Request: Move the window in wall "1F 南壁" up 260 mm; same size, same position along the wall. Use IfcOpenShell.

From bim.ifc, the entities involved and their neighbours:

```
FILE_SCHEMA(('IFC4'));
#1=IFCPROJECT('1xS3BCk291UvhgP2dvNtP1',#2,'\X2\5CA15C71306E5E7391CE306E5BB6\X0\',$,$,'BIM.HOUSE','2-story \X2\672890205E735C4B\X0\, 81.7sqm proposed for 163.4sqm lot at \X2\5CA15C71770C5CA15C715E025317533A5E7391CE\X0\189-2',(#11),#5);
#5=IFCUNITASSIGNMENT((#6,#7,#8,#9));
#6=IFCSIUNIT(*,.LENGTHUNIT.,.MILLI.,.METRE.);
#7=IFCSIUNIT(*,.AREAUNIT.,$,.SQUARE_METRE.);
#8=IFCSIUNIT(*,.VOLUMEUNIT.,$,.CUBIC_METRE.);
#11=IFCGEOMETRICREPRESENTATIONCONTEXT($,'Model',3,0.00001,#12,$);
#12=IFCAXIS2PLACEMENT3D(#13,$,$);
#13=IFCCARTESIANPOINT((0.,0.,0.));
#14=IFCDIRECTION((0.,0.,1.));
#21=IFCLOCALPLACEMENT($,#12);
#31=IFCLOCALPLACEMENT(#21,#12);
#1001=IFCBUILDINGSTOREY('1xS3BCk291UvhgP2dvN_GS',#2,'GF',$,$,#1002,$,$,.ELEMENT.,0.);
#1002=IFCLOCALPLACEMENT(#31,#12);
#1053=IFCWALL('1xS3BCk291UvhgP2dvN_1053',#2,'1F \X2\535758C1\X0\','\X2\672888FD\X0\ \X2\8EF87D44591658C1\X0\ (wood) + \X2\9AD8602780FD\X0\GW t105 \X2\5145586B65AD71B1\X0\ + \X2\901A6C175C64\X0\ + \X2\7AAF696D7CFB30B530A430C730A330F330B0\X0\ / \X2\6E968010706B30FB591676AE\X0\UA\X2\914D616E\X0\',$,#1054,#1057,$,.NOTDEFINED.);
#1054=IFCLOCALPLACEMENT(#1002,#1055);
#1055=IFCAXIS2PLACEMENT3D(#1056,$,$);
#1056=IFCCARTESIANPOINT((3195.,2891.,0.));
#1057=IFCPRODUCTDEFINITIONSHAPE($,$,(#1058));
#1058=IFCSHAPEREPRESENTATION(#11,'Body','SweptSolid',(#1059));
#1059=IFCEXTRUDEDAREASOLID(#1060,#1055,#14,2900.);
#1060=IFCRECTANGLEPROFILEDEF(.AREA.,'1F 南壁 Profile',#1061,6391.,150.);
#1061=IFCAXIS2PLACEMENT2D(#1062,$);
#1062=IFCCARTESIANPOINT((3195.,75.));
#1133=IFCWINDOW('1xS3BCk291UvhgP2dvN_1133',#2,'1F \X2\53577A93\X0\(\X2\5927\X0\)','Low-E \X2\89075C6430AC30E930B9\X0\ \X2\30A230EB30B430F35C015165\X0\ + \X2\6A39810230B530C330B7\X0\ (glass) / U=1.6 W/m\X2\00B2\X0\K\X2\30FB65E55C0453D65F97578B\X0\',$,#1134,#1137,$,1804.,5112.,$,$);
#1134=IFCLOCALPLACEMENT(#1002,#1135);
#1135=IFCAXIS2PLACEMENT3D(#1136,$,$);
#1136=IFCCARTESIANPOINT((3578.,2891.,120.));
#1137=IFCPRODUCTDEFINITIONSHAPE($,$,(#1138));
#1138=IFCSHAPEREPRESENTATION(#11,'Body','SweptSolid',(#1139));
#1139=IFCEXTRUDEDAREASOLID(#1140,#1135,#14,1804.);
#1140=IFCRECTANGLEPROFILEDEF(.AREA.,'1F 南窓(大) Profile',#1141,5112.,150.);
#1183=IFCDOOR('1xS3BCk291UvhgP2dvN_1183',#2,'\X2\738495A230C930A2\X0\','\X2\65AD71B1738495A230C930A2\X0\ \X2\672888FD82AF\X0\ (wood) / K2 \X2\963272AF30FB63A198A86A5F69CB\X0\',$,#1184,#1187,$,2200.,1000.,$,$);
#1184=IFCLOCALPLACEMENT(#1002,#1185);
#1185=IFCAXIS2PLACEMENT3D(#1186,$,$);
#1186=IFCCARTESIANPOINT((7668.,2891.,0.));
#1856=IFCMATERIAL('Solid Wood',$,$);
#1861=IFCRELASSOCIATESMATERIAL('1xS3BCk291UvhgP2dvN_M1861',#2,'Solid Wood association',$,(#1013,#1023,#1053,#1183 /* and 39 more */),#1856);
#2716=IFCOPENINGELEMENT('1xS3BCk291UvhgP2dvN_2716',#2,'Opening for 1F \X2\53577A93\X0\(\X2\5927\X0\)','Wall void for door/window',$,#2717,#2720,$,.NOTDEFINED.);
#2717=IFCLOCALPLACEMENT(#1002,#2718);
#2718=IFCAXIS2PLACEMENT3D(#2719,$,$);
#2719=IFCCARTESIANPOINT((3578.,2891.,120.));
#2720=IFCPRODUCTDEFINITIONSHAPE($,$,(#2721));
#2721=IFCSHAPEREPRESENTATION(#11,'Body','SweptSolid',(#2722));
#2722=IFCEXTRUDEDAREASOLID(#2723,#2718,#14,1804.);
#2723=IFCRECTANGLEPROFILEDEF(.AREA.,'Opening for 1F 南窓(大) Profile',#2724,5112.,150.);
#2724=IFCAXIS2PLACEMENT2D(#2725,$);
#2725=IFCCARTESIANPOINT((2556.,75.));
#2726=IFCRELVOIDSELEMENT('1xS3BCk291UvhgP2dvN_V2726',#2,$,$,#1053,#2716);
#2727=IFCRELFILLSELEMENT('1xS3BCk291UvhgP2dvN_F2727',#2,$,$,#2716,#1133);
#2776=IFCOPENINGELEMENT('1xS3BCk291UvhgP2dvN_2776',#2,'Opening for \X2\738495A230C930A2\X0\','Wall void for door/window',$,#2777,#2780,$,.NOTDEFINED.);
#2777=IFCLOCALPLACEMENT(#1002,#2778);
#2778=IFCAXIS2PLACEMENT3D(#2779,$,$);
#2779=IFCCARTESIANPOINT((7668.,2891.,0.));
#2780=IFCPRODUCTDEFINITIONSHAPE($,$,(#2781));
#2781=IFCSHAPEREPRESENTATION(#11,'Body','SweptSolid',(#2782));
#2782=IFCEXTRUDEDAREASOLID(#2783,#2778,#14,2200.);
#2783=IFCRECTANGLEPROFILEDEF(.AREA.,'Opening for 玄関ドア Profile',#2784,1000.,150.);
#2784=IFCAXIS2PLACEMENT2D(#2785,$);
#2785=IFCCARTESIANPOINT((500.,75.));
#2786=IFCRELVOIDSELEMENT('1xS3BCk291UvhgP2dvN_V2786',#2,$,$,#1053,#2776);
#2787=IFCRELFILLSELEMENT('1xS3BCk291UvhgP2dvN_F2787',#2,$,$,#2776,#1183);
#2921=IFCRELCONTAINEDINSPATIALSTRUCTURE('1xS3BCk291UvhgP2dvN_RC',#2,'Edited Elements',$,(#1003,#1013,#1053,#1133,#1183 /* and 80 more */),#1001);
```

```python
import numpy as np
import ifcopenshell
import ifcopenshell.api.geometry
import ifcopenshell.util.placement
import ifcopenshell.util.unit

model = ifcopenshell.open("bim.ifc")
unit_scale = ifcopenshell.util.unit.calculate_unit_scale(model)

window = model.by_guid("1xS3BCk291UvhgP2dvN_1133")
opening = window.FillsVoids[0].RelatingOpeningElement
dz = 0.26 / unit_scale

shift = np.array([0.0, 0.0, dz])
# The window is not placed relative to its opening, so move both.
for product in (opening, window):
    matrix = ifcopenshell.util.placement.get_local_placement(product.ObjectPlacement)
    matrix[:3, 3] += shift
    ifcopenshell.api.geometry.edit_object_placement(model, product=product, matrix=matrix, is_si=False)

print(f"moved by {dz * unit_scale:+.3f} m")

model.write("bim-out.ifc")
```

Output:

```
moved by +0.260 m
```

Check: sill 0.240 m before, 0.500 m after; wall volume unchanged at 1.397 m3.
